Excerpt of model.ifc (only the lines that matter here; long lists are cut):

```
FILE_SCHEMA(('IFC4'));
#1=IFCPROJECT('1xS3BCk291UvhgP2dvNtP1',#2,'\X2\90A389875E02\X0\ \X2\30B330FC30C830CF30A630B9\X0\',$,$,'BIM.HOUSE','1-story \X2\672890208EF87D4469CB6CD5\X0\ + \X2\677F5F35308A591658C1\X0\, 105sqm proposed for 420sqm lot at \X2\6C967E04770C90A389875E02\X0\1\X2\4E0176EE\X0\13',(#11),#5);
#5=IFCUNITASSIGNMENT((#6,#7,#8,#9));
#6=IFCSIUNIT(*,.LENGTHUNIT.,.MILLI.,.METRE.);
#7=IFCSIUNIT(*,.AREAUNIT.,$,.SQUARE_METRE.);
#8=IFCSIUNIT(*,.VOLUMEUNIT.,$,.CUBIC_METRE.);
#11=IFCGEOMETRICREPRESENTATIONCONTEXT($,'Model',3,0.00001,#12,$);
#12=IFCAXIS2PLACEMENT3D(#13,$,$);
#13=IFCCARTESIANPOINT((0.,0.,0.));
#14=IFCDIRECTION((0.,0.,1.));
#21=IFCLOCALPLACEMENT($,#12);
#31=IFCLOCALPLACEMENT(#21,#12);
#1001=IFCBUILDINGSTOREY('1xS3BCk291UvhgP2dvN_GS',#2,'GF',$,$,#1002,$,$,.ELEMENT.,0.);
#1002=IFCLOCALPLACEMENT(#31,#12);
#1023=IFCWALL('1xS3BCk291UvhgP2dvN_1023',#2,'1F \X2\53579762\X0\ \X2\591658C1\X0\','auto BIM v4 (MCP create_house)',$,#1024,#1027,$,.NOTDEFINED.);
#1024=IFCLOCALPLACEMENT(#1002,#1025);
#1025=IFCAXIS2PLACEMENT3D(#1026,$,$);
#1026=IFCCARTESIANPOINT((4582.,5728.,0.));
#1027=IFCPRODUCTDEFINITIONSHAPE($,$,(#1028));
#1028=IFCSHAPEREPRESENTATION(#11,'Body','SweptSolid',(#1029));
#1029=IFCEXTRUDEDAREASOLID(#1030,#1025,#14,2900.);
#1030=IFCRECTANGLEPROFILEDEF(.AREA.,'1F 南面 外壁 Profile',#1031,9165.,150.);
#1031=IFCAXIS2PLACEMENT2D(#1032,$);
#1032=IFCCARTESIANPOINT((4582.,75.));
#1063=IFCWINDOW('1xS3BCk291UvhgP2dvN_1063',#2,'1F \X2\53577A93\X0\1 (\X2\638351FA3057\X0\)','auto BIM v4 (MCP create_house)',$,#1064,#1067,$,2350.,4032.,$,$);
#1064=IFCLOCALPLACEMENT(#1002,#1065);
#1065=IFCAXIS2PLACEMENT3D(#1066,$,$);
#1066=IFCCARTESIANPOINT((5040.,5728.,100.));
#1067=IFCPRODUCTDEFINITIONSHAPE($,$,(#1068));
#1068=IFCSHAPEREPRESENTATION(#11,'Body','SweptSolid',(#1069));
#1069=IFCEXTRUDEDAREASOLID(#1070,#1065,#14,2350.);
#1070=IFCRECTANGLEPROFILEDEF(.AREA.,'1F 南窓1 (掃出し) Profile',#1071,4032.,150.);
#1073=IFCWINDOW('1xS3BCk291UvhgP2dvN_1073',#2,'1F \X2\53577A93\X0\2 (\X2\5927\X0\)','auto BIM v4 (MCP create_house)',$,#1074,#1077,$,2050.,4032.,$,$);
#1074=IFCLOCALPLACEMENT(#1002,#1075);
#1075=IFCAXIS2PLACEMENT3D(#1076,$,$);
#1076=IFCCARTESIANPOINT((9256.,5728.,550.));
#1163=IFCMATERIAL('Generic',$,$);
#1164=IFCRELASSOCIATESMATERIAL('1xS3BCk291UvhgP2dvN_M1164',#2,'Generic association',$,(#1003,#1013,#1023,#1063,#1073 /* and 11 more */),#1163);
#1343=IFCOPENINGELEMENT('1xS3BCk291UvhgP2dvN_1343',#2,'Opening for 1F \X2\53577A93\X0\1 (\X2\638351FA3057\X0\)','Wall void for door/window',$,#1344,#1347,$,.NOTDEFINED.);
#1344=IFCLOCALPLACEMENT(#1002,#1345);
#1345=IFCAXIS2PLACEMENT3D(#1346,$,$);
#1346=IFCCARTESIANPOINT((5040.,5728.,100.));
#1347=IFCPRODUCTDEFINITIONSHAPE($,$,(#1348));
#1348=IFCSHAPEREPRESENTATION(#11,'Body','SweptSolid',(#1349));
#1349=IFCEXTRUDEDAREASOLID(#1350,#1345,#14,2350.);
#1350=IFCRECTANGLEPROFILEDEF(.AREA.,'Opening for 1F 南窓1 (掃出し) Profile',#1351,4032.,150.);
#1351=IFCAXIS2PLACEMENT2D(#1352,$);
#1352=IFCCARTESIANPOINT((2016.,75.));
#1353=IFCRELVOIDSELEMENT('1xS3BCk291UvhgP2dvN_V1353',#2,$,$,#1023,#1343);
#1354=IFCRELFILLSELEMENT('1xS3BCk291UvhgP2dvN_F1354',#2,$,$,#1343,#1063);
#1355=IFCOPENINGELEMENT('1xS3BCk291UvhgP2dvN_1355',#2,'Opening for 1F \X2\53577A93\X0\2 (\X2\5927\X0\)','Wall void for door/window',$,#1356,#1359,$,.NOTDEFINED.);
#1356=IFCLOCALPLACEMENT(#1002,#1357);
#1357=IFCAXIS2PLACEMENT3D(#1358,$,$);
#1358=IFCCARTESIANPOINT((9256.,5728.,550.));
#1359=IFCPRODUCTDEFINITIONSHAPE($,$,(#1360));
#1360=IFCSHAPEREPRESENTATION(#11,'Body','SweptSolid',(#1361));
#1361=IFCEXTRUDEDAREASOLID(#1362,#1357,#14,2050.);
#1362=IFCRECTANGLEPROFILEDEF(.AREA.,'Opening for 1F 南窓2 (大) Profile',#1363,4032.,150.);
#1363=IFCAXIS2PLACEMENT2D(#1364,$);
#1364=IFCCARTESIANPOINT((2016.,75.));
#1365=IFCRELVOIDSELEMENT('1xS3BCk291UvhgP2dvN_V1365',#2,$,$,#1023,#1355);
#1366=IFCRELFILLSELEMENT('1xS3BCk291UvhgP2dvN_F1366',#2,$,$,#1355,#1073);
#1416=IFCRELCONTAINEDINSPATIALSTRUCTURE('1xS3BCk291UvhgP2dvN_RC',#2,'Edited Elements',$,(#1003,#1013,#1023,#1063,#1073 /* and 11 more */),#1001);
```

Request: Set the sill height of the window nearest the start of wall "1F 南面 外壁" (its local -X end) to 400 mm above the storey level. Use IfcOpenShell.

```python
import numpy as np
import ifcopenshell
import ifcopenshell.api.geometry
import ifcopenshell.geom
import ifcopenshell.util.element
import ifcopenshell.util.placement
import ifcopenshell.util.shape
import ifcopenshell.util.unit

model = ifcopenshell.open("model.ifc")
unit_scale = ifcopenshell.util.unit.calculate_unit_scale(model)

window = model.by_id(1063)
opening = window.FillsVoids[0].RelatingOpeningElement
storey = ifcopenshell.util.element.get_container(window, ifc_class="IfcBuildingStorey")
level = ifcopenshell.util.placement.get_local_placement(storey.ObjectPlacement)[2, 3]

# The opening's origin need not be at the sill, so measure its lowest point.
shape = ifcopenshell.geom.create_shape(ifcopenshell.geom.settings(), opening)
bottom = ifcopenshell.util.shape.get_shape_bottom_elevation(shape, shape.geometry) / unit_scale
dz = level + 0.4 / unit_scale - bottom

shift = np.array([0.0, 0.0, dz])
# The window is not placed relative to its opening, so move both.
for product in (opening, window):
    matrix = ifcopenshell.util.placement.get_local_placement(product.ObjectPlacement)
    matrix[:3, 3] += shift
    ifcopenshell.api.geometry.edit_object_placement(model, product=product, matrix=matrix, is_si=False)

print(f"moved by {dz * unit_scale:+.3f} m")

model.write("model_rev.ifc")
```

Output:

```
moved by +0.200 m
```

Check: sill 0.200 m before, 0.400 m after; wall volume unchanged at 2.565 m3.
